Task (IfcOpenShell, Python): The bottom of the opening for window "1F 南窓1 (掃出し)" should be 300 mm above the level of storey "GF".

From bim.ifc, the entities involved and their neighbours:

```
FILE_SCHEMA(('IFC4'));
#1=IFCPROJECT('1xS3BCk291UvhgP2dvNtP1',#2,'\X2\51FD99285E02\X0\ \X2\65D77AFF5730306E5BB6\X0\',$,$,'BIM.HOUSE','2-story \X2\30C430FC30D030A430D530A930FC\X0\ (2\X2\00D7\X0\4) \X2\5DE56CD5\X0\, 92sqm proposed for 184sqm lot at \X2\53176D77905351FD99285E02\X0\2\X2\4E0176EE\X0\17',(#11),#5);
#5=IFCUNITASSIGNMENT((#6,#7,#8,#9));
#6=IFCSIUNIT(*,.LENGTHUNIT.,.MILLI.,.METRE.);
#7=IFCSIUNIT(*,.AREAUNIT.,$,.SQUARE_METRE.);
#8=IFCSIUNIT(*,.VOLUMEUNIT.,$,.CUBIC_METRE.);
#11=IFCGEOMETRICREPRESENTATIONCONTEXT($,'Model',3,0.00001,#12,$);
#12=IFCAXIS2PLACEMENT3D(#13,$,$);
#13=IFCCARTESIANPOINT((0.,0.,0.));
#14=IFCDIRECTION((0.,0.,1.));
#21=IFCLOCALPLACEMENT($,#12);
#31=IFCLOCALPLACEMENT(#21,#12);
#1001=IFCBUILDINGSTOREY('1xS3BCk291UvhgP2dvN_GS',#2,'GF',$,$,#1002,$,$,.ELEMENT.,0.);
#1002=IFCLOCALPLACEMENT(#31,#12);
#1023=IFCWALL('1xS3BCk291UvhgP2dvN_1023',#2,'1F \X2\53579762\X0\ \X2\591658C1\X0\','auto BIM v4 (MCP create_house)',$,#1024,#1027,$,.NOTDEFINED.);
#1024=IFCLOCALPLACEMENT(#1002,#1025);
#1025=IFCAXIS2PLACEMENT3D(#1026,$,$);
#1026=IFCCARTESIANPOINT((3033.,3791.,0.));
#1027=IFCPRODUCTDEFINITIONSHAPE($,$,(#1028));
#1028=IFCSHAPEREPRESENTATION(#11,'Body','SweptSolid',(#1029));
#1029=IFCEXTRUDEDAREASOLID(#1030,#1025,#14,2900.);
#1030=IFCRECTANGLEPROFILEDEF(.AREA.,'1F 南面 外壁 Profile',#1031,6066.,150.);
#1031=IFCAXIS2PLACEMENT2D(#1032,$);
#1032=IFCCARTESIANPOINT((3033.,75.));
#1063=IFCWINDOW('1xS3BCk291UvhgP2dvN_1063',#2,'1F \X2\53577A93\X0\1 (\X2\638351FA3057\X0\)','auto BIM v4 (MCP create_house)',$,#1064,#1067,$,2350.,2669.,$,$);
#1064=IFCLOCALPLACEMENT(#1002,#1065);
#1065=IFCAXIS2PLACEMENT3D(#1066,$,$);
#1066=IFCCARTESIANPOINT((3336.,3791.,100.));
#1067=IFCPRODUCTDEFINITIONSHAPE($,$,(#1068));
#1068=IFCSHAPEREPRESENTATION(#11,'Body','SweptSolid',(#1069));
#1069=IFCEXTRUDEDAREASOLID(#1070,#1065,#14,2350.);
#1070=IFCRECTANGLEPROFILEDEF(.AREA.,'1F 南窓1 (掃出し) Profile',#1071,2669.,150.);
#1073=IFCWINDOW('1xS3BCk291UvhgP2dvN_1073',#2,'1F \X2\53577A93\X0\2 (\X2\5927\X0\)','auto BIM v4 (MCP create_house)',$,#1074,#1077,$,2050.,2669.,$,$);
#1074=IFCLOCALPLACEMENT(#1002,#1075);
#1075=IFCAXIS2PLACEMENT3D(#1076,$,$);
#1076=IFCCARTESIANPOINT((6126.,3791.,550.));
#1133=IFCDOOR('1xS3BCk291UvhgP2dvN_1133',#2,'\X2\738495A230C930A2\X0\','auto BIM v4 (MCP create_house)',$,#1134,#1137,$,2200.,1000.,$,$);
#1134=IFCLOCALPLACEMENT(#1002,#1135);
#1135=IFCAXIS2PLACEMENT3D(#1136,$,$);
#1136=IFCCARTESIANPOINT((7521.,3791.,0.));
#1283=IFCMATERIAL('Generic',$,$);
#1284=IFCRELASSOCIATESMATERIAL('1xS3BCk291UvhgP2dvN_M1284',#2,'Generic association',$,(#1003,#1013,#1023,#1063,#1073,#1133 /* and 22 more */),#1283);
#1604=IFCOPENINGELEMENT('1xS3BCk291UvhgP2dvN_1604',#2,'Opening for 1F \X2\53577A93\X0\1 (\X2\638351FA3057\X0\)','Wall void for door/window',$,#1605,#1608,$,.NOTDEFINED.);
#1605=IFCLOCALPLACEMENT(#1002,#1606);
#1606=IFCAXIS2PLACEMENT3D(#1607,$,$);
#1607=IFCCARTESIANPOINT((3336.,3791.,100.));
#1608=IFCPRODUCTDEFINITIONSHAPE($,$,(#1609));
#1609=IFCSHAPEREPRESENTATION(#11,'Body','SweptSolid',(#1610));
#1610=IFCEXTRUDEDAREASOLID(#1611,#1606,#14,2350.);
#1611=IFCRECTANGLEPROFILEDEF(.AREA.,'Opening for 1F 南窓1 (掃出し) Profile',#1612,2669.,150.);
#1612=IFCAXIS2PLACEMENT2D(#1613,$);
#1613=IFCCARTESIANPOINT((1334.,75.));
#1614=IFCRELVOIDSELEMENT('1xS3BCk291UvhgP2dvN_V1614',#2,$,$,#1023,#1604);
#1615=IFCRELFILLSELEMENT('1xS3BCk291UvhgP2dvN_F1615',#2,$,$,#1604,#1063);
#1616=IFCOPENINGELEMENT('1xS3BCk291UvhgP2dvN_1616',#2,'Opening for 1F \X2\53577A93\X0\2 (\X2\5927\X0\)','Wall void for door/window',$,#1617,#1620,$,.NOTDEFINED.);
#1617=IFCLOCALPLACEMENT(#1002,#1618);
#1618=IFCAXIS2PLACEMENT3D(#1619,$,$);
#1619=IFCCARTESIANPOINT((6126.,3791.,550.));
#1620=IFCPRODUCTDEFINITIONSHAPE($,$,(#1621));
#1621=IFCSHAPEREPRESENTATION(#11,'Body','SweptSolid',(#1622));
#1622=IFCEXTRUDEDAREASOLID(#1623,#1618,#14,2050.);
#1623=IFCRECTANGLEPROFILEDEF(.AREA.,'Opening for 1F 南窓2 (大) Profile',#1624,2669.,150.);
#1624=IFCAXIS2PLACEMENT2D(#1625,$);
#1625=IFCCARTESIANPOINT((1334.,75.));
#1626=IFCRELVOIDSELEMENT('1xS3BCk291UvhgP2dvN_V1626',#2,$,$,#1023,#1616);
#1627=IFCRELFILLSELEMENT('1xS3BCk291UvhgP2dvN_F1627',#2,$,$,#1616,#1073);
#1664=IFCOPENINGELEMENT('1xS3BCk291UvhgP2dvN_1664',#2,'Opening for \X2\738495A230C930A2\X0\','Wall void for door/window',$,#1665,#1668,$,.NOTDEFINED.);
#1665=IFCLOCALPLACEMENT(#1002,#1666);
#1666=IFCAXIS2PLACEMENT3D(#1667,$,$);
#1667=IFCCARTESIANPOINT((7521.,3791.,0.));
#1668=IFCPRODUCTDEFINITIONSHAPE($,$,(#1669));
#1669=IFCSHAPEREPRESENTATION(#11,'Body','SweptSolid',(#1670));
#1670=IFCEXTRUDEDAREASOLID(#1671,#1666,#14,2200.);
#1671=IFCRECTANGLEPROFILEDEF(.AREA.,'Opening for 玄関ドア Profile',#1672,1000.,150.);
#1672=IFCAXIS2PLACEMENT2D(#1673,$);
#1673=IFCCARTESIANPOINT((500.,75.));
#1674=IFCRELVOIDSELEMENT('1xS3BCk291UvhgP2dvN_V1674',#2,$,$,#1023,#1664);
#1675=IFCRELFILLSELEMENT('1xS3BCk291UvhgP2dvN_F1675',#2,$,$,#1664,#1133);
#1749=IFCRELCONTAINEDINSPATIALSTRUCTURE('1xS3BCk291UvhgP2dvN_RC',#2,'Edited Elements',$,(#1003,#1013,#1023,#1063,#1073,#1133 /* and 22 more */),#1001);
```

```python
import numpy as np
import ifcopenshell
import ifcopenshell.api.geometry
import ifcopenshell.geom
import ifcopenshell.util.element
import ifcopenshell.util.placement
import ifcopenshell.util.shape
import ifcopenshell.util.unit

model = ifcopenshell.open("bim.ifc")
unit_scale = ifcopenshell.util.unit.calculate_unit_scale(model)

window = model.by_guid("1xS3BCk291UvhgP2dvN_1063")
opening = window.FillsVoids[0].RelatingOpeningElement
storey = ifcopenshell.util.element.get_container(window, ifc_class="IfcBuildingStorey")
level = ifcopenshell.util.placement.get_local_placement(storey.ObjectPlacement)[2, 3]

# The opening's origin need not be at the sill, so measure its lowest point.
shape = ifcopenshell.geom.create_shape(ifcopenshell.geom.settings(), opening)
bottom = ifcopenshell.util.shape.get_shape_bottom_elevation(shape, shape.geometry) / unit_scale
dz = level + 0.3 / unit_scale - bottom

shift = np.array([0.0, 0.0, dz])
# The window is not placed relative to its opening, so move both.
for product in (opening, window):
    matrix = ifcopenshell.util.placement.get_local_placement(product.ObjectPlacement)
    matrix[:3, 3] += shift
    ifcopenshell.api.geometry.edit_object_placement(model, product=product, matrix=matrix, is_si=False)

print(f"moved by {dz * unit_scale:+.3f} m")

model.write("bim_edited.ifc")
```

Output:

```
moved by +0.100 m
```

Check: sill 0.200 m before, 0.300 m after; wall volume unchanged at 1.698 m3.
